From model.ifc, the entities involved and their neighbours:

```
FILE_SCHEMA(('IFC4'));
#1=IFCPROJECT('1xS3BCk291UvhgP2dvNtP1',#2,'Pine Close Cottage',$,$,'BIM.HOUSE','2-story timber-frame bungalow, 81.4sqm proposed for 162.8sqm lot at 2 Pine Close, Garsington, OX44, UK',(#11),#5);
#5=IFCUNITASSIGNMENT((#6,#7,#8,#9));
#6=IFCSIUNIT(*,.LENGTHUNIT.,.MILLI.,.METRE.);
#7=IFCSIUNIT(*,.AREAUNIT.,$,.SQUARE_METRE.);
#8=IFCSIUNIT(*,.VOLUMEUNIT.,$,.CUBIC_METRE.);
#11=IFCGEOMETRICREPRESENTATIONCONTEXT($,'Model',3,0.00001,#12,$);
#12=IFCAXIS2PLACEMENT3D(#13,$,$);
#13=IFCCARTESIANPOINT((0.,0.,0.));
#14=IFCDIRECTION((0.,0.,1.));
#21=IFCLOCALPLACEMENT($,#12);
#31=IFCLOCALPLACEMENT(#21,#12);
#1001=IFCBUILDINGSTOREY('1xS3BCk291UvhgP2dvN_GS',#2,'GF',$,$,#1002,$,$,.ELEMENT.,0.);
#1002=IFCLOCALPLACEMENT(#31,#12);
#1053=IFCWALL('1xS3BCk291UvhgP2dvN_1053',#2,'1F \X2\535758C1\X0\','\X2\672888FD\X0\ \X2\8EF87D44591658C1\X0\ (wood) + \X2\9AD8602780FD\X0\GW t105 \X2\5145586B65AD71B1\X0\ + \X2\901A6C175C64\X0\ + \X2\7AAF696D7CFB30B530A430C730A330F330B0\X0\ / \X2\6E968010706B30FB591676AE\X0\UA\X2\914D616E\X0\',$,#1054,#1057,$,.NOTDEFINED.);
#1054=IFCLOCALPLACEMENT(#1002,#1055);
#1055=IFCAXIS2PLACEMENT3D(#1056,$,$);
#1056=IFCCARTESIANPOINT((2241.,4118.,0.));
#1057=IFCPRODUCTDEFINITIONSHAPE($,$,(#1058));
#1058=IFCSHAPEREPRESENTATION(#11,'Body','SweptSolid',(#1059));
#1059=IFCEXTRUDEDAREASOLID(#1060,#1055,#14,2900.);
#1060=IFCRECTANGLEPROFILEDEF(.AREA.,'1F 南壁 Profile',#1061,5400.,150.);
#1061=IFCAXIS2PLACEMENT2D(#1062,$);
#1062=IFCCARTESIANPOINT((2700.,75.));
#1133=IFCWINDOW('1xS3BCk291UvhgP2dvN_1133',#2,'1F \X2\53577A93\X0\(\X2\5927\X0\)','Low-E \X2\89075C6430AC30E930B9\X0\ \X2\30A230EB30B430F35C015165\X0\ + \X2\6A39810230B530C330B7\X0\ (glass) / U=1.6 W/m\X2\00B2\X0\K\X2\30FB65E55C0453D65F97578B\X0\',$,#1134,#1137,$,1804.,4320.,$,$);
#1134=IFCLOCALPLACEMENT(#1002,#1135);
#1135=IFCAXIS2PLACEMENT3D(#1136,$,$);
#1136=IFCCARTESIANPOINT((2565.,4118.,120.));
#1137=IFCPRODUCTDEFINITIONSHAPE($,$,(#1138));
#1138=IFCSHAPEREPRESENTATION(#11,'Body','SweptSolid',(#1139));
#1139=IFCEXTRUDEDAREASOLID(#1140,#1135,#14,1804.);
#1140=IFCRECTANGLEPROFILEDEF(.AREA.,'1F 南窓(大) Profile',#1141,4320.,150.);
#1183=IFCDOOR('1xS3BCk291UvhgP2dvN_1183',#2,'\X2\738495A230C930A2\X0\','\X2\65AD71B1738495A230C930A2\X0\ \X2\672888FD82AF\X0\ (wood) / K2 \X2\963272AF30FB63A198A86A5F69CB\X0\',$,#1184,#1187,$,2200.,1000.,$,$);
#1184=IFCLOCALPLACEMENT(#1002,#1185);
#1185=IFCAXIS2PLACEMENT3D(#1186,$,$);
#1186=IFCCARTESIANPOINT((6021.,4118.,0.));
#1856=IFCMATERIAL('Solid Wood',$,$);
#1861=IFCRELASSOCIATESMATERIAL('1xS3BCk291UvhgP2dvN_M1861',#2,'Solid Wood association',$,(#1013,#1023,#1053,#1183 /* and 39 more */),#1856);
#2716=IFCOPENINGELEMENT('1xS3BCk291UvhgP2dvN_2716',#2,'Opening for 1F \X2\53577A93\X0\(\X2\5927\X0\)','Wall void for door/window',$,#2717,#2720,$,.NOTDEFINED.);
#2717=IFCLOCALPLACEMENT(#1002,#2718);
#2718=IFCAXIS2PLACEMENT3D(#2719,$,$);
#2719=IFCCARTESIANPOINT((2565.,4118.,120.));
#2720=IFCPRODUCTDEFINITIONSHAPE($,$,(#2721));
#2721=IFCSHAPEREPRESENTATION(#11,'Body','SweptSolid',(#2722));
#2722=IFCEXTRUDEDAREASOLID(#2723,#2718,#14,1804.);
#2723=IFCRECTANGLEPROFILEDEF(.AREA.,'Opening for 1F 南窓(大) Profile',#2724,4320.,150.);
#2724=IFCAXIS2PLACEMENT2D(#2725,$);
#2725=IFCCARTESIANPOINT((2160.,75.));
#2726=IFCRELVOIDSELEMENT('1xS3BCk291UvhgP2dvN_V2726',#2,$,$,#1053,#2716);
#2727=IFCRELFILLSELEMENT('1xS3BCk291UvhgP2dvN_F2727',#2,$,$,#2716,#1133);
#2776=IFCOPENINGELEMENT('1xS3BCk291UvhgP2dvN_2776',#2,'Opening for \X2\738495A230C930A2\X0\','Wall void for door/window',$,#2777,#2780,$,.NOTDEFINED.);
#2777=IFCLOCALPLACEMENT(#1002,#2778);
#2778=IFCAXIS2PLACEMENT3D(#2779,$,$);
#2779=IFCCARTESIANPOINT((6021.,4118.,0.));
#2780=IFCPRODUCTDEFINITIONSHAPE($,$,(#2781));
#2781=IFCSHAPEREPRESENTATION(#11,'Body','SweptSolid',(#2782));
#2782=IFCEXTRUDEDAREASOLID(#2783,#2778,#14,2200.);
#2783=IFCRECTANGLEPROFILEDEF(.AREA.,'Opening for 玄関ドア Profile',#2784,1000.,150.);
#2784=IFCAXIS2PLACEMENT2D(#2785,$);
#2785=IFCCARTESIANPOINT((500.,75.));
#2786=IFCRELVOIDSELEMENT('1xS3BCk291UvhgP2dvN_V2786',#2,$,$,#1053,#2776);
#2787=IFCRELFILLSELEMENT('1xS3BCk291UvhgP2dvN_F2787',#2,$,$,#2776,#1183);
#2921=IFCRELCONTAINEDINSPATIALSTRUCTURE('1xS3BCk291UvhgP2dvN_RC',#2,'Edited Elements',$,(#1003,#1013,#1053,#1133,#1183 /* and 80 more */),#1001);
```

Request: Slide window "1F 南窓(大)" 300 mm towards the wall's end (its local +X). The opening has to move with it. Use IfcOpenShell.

```python
import ifcopenshell
import ifcopenshell.api.geometry
import ifcopenshell.util.placement
import ifcopenshell.util.unit

model = ifcopenshell.open("model.ifc")
unit_scale = ifcopenshell.util.unit.calculate_unit_scale(model)

window = model.by_id(1133)
opening = window.FillsVoids[0].RelatingOpeningElement
wall = opening.VoidsElements[0].RelatingBuildingElement

wall_matrix = ifcopenshell.util.placement.get_local_placement(wall.ObjectPlacement)
shift = wall_matrix[:3, 0] * 0.3 / unit_scale
before = ifcopenshell.util.placement.get_local_placement(window.ObjectPlacement)[:3, 3].copy()

# The window is not placed relative to its opening, so move both.
for product in (opening, window):
    matrix = ifcopenshell.util.placement.get_local_placement(product.ObjectPlacement)
    matrix[:3, 3] += shift
    ifcopenshell.api.geometry.edit_object_placement(model, product=product, matrix=matrix, is_si=False)

after = ifcopenshell.util.placement.get_local_placement(window.ObjectPlacement)[:3, 3]
print("window moved by", (after - before).round(3) + 0.0)

model.write("model_v2.ifc")
```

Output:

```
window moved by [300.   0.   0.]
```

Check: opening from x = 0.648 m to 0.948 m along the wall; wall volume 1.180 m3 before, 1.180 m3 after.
